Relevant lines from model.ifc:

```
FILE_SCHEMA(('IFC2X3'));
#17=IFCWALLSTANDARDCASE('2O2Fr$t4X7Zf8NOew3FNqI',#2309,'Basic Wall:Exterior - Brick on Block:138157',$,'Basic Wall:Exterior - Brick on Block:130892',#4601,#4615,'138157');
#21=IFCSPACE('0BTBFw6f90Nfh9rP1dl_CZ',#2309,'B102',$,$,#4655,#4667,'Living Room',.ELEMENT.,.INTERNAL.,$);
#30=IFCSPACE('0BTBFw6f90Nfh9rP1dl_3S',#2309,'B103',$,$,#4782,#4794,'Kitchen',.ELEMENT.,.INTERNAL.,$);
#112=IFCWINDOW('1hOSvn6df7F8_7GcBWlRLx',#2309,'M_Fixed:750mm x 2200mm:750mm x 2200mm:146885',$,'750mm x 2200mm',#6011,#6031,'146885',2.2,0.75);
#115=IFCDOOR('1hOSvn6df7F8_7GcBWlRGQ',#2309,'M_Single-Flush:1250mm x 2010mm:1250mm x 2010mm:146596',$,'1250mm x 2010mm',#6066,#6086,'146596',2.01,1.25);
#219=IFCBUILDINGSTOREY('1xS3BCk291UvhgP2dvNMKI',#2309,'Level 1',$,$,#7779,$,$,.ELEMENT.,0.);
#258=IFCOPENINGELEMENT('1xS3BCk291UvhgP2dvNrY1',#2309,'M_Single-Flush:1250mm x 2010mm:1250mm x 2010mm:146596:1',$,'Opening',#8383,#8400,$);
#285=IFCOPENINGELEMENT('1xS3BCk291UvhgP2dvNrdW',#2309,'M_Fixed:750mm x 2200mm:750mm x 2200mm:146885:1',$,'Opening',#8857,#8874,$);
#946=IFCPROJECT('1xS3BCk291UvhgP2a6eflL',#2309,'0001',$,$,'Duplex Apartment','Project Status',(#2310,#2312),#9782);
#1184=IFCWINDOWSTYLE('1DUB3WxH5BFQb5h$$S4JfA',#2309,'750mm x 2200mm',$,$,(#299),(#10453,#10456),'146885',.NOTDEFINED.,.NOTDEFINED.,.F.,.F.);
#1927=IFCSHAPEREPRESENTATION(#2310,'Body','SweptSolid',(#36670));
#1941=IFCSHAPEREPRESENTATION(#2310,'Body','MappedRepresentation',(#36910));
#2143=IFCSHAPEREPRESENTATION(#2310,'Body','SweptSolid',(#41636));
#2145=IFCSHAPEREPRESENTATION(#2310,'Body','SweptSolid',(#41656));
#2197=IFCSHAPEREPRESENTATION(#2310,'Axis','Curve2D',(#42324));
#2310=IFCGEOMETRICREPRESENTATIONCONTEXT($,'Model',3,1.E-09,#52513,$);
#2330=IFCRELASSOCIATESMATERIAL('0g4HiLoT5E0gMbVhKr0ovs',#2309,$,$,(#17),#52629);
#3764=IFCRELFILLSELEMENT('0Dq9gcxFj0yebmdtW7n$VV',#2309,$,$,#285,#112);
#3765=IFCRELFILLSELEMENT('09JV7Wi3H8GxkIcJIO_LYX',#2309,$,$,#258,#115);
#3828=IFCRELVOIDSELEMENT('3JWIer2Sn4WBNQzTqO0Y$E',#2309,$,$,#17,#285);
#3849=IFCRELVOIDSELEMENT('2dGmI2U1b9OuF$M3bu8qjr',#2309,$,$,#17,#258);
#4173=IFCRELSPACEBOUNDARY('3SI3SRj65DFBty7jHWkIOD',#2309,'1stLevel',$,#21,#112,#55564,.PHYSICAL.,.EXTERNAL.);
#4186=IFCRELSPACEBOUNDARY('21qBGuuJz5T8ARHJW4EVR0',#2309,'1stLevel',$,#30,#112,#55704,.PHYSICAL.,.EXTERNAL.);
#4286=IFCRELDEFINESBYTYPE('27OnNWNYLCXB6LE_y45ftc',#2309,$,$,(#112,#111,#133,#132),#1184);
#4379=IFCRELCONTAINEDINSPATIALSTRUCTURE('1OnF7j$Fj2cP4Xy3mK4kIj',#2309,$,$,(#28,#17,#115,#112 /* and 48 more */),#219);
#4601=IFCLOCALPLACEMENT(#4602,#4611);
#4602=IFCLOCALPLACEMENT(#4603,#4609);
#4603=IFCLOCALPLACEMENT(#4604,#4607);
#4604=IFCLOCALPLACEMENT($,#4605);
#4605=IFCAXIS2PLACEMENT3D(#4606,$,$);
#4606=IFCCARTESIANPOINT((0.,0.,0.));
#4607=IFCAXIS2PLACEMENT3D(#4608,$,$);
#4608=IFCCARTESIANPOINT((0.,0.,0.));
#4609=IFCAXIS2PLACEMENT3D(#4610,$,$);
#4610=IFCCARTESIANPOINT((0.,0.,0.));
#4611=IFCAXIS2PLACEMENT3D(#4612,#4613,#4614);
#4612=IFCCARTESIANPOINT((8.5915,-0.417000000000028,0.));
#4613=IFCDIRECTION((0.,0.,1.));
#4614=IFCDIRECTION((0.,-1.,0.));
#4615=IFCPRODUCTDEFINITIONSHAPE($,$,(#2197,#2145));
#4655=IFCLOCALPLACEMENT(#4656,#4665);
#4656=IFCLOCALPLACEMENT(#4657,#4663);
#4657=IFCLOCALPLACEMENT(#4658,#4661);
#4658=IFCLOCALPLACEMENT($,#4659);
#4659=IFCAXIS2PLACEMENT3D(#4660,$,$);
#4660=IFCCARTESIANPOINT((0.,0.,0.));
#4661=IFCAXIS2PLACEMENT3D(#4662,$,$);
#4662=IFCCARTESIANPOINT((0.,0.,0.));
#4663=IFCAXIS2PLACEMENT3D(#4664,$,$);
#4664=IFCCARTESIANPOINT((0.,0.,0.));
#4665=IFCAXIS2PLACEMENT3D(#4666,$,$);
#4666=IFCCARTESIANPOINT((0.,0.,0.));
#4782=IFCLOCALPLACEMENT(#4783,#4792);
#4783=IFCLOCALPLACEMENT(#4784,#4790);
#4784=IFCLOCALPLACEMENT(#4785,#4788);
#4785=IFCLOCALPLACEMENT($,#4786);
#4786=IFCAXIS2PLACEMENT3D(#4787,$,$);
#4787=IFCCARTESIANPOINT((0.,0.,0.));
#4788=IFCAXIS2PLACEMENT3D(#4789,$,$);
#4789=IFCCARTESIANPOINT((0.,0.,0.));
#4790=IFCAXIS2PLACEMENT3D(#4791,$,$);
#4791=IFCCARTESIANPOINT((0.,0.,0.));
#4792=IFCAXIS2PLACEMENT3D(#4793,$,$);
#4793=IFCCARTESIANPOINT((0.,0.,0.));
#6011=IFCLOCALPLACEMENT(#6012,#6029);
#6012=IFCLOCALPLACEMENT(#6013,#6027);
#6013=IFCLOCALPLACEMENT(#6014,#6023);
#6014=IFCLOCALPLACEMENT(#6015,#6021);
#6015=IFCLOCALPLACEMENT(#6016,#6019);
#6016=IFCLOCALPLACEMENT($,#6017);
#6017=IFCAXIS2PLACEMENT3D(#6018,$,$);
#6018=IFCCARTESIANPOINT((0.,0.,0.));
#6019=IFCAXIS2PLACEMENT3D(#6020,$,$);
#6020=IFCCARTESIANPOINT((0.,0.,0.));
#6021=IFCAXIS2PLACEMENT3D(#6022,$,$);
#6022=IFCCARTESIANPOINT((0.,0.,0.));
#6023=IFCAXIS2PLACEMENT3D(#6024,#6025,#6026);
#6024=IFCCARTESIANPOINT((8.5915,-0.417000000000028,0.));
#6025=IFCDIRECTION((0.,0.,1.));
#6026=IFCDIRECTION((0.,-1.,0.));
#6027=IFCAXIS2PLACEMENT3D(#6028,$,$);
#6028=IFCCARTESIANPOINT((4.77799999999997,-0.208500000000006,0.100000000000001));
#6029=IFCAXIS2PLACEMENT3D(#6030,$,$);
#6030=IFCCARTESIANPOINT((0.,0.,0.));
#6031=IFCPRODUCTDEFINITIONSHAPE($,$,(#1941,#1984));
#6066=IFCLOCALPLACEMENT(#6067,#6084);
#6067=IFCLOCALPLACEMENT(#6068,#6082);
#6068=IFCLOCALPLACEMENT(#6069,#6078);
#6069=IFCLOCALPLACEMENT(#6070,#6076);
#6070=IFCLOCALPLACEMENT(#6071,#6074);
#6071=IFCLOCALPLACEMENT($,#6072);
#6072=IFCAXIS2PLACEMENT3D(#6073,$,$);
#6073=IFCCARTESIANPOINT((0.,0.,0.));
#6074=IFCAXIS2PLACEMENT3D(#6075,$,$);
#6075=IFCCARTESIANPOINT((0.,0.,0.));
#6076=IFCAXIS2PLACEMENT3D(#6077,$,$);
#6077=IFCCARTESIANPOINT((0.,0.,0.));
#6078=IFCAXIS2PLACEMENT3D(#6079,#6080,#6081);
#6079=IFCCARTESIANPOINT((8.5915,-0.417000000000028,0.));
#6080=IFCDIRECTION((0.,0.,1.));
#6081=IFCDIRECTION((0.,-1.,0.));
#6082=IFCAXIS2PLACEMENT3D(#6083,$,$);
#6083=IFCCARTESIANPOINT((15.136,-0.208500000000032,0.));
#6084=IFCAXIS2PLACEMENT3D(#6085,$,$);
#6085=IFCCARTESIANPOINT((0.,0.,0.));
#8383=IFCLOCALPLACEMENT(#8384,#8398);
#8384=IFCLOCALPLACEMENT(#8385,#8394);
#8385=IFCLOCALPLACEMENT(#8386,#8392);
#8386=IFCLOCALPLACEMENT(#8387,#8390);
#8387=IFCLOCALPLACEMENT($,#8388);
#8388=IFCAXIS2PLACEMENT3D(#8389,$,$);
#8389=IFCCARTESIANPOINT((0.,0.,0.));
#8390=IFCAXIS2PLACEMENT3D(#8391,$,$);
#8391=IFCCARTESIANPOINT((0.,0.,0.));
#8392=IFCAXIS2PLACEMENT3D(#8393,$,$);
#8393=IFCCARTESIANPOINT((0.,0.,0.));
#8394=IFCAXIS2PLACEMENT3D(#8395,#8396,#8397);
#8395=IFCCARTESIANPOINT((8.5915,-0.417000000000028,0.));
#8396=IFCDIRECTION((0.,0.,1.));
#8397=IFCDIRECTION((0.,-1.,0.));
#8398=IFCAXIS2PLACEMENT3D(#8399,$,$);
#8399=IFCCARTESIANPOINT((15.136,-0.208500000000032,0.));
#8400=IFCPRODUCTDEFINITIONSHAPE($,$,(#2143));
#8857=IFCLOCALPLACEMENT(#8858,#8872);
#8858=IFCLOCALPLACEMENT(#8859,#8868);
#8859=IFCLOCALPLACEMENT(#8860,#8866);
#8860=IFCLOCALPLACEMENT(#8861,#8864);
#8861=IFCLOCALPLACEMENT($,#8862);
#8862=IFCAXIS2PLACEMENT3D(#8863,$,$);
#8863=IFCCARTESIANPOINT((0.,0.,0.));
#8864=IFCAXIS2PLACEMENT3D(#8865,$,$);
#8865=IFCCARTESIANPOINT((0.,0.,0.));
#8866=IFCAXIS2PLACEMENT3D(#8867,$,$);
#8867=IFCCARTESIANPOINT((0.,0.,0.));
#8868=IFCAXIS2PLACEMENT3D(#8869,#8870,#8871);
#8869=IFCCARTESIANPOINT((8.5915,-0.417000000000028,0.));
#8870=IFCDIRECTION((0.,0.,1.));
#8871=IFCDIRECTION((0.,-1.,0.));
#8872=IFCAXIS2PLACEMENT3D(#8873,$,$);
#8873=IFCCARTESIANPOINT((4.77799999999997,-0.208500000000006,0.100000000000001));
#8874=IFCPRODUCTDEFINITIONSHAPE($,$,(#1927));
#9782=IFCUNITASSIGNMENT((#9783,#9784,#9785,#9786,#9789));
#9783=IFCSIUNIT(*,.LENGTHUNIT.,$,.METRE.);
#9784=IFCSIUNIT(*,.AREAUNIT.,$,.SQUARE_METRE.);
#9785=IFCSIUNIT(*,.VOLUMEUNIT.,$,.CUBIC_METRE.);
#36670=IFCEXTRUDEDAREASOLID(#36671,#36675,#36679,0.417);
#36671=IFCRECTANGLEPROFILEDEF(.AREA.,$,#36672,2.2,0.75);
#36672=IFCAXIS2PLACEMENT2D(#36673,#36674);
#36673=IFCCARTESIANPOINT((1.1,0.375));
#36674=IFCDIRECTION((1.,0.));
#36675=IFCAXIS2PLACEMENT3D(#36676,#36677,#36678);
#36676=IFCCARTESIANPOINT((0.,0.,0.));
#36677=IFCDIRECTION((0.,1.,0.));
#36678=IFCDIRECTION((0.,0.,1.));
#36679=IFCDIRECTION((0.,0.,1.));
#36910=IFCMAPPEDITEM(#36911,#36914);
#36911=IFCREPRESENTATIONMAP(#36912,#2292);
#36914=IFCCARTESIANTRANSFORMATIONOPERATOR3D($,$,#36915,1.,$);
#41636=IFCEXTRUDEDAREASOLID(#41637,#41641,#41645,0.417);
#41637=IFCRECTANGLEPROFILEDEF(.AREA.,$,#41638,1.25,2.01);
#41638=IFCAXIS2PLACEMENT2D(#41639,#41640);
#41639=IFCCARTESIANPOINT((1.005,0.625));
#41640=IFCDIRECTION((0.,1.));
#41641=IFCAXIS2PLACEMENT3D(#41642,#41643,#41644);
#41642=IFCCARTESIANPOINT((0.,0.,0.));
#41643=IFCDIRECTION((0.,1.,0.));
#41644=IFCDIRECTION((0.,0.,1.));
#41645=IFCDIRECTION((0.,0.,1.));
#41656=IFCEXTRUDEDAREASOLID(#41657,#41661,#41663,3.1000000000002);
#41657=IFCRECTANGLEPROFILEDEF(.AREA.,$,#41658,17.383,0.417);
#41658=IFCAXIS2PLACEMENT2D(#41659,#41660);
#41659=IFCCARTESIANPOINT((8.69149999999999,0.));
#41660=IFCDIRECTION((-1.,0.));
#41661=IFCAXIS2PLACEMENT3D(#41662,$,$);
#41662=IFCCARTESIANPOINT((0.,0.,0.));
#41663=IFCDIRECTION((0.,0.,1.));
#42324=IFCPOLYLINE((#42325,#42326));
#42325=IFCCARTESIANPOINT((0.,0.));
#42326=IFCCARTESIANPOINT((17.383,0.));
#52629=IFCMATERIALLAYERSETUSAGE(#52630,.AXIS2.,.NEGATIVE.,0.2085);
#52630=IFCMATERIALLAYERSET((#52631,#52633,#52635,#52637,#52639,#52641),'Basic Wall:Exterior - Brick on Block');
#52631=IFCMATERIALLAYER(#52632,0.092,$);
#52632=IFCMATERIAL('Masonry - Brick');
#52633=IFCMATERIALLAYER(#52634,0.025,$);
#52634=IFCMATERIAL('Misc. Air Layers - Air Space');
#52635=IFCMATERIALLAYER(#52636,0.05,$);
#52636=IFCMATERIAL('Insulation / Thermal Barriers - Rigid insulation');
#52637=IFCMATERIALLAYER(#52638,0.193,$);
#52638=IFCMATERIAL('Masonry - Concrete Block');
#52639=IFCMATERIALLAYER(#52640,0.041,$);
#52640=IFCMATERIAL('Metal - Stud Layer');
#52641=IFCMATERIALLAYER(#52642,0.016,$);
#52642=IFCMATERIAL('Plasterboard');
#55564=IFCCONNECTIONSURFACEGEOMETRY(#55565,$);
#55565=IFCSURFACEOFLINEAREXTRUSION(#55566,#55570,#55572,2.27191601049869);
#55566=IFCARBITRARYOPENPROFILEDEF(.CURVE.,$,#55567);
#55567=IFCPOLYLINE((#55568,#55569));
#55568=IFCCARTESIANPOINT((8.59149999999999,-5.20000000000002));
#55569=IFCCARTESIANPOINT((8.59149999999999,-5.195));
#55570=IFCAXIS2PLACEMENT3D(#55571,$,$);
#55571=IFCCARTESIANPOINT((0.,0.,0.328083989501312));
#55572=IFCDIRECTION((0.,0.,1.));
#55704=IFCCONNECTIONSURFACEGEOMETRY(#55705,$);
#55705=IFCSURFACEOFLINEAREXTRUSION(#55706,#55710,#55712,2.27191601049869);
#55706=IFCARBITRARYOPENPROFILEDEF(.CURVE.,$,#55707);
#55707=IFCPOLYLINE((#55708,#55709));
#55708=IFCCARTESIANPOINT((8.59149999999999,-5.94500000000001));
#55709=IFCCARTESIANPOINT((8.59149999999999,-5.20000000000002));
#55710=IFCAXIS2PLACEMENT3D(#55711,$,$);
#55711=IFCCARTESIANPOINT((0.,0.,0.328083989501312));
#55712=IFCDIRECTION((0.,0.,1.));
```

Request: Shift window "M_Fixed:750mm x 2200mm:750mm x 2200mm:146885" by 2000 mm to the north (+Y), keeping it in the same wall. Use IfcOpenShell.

```python
import numpy as np
import ifcopenshell
import ifcopenshell.api.geometry
import ifcopenshell.util.placement

model = ifcopenshell.open("model.ifc")

window = model.by_guid("1hOSvn6df7F8_7GcBWlRLx")
opening = window.FillsVoids[0].RelatingOpeningElement
wall = opening.VoidsElements[0].RelatingBuildingElement

wall_matrix = ifcopenshell.util.placement.get_local_placement(wall.ObjectPlacement)
shift = wall_matrix[:3, 0] * -2.0
before = ifcopenshell.util.placement.get_local_placement(window.ObjectPlacement)[:3, 3].copy()

# The window is not placed relative to its opening, so move both.
for product in (opening, window):
    matrix = ifcopenshell.util.placement.get_local_placement(product.ObjectPlacement)
    matrix[:3, 3] += shift
    ifcopenshell.api.geometry.edit_object_placement(model, product=product, matrix=matrix, is_si=False)

# Space boundary surfaces are stored in each space's coordinates; move them too.
for rel in window.ProvidesBoundaries:
    if not rel.ConnectionGeometry:
        continue
    surface = rel.ConnectionGeometry.SurfaceOnRelatingElement
    space_matrix = ifcopenshell.util.placement.get_local_placement(rel.RelatingSpace.ObjectPlacement)
    point = np.array(surface.Position.Location.Coordinates) + space_matrix[:3, :3].T @ shift
    surface.Position = model.createIfcAxis2Placement3D(
        model.createIfcCartesianPoint(point.tolist()), surface.Position.Axis, surface.Position.RefDirection
    )

after = ifcopenshell.util.placement.get_local_placement(window.ObjectPlacement)[:3, 3]
print("window moved by", (after - before).round(3) + 0.0)

model.write("model_edited.ifc")
```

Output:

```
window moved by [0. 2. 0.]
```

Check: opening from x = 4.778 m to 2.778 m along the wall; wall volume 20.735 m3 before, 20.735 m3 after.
